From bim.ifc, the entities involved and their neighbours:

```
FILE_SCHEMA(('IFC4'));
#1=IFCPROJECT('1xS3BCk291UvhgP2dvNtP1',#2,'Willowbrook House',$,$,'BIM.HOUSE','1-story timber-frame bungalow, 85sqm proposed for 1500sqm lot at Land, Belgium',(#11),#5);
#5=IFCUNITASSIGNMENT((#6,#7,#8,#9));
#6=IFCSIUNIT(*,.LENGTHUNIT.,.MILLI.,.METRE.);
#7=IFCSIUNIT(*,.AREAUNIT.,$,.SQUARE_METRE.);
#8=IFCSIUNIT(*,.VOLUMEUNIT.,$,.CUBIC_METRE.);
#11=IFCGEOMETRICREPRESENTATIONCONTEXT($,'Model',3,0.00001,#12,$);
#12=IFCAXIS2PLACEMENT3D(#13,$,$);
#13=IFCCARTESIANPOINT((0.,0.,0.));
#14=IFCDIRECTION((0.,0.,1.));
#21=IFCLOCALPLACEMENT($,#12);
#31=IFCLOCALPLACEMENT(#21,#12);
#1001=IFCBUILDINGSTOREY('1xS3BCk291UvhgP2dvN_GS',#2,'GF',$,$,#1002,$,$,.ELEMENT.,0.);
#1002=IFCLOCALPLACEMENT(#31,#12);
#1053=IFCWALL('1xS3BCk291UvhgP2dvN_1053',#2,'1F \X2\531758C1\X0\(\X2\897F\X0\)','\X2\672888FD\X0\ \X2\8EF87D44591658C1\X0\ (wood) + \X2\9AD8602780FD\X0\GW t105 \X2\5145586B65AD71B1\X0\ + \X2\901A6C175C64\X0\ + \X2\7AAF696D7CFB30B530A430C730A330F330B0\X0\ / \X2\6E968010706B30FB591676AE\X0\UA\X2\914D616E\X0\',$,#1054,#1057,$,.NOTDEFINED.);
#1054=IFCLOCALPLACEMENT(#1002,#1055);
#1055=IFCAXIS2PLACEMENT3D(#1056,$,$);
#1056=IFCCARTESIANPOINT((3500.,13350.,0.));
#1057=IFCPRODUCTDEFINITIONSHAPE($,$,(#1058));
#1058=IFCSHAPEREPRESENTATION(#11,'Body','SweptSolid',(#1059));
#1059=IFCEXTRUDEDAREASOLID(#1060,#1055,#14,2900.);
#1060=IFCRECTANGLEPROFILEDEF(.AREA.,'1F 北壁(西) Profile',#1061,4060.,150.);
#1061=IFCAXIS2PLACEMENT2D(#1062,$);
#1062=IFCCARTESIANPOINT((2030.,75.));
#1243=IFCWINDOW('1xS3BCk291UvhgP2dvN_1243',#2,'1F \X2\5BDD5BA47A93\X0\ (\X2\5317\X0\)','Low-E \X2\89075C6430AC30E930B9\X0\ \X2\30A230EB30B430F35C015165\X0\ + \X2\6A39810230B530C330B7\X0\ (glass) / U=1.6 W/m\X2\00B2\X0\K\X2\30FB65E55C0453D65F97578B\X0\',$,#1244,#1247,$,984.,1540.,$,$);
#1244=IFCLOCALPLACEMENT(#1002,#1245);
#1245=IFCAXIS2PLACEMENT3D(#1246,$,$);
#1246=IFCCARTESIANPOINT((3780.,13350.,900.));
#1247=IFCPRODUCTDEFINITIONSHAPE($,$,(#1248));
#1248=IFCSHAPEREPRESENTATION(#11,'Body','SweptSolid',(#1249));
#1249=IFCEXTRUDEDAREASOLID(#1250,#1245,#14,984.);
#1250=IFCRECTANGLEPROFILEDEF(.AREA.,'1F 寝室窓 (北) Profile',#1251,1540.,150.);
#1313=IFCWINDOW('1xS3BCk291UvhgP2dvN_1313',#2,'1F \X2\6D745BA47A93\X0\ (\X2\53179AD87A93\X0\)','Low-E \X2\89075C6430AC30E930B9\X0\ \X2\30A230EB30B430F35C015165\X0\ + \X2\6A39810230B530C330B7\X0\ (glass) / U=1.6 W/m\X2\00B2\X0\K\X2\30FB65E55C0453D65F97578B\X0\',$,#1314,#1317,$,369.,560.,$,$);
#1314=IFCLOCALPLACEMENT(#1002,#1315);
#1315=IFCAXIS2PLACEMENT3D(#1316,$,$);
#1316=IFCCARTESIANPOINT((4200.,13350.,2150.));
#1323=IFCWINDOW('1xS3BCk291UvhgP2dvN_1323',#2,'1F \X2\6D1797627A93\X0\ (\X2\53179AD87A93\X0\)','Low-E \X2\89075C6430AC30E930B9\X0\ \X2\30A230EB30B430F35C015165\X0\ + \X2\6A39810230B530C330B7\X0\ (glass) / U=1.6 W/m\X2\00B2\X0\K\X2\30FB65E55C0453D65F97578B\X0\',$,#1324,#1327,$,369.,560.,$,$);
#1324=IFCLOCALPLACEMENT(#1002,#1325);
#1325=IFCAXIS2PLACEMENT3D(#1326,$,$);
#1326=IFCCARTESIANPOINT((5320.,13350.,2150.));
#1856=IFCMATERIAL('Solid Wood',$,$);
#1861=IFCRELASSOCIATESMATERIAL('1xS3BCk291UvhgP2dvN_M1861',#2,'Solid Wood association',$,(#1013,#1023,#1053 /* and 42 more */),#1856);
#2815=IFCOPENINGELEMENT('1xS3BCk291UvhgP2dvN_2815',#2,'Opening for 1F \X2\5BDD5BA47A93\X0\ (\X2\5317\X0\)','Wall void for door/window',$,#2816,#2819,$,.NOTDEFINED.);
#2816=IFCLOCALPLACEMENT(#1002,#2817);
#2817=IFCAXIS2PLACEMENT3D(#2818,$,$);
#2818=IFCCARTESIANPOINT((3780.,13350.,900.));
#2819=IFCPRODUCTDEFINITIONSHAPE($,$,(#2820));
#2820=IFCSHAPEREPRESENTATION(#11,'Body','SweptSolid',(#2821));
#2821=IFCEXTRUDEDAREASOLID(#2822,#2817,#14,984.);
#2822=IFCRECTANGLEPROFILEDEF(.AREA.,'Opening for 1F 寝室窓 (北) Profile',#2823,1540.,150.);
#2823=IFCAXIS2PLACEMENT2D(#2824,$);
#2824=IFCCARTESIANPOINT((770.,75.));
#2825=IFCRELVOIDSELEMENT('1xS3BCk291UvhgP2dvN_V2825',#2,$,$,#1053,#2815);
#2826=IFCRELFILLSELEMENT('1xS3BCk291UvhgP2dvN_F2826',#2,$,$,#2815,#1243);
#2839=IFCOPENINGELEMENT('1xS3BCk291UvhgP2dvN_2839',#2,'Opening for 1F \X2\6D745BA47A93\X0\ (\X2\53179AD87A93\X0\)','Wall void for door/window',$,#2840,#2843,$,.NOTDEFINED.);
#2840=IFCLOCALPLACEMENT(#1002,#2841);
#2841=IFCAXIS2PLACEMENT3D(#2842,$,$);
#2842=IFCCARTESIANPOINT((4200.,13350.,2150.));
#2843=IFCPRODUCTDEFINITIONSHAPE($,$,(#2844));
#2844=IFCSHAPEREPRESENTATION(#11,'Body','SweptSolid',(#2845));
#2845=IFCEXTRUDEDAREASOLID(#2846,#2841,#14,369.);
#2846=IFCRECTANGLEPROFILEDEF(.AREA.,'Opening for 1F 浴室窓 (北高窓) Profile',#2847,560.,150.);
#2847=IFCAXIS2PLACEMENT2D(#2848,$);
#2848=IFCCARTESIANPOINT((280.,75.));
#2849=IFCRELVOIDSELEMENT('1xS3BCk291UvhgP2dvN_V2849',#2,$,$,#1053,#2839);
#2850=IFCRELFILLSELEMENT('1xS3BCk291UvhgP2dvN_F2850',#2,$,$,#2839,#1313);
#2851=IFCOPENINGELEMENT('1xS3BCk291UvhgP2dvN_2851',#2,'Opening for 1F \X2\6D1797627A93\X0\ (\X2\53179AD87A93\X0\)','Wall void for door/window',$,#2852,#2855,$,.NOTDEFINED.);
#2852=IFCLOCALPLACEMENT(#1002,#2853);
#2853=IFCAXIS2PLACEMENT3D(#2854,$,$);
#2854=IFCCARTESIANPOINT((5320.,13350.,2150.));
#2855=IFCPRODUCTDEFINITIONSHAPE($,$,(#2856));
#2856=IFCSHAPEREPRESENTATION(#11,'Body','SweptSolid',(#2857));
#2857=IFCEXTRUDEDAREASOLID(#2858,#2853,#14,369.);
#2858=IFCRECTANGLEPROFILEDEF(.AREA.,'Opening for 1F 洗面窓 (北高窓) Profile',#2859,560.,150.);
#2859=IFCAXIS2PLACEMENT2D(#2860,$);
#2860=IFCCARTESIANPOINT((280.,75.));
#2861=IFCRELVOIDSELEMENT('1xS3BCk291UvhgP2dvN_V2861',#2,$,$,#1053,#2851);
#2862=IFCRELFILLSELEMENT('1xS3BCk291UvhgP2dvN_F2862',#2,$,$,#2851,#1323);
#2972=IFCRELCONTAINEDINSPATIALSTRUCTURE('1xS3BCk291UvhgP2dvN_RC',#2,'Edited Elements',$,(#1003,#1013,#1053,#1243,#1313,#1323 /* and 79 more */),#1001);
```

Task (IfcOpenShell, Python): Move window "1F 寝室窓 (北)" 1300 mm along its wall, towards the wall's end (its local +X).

```python
import ifcopenshell
import ifcopenshell.api.geometry
import ifcopenshell.util.placement
import ifcopenshell.util.unit

model = ifcopenshell.open("bim.ifc")
unit_scale = ifcopenshell.util.unit.calculate_unit_scale(model)

window = model.by_guid("1xS3BCk291UvhgP2dvN_1243")
opening = window.FillsVoids[0].RelatingOpeningElement
wall = opening.VoidsElements[0].RelatingBuildingElement

wall_matrix = ifcopenshell.util.placement.get_local_placement(wall.ObjectPlacement)
shift = wall_matrix[:3, 0] * 1.3 / unit_scale
before = ifcopenshell.util.placement.get_local_placement(window.ObjectPlacement)[:3, 3].copy()

# The window is not placed relative to its opening, so move both.
for product in (opening, window):
    matrix = ifcopenshell.util.placement.get_local_placement(product.ObjectPlacement)
    matrix[:3, 3] += shift
    ifcopenshell.api.geometry.edit_object_placement(model, product=product, matrix=matrix, is_si=False)

after = ifcopenshell.util.placement.get_local_placement(window.ObjectPlacement)[:3, 3]
print("window moved by", (after - before).round(3) + 0.0)

model.write("bim_v2.ifc")
```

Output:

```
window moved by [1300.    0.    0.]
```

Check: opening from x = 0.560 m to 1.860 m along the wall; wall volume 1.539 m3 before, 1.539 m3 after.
